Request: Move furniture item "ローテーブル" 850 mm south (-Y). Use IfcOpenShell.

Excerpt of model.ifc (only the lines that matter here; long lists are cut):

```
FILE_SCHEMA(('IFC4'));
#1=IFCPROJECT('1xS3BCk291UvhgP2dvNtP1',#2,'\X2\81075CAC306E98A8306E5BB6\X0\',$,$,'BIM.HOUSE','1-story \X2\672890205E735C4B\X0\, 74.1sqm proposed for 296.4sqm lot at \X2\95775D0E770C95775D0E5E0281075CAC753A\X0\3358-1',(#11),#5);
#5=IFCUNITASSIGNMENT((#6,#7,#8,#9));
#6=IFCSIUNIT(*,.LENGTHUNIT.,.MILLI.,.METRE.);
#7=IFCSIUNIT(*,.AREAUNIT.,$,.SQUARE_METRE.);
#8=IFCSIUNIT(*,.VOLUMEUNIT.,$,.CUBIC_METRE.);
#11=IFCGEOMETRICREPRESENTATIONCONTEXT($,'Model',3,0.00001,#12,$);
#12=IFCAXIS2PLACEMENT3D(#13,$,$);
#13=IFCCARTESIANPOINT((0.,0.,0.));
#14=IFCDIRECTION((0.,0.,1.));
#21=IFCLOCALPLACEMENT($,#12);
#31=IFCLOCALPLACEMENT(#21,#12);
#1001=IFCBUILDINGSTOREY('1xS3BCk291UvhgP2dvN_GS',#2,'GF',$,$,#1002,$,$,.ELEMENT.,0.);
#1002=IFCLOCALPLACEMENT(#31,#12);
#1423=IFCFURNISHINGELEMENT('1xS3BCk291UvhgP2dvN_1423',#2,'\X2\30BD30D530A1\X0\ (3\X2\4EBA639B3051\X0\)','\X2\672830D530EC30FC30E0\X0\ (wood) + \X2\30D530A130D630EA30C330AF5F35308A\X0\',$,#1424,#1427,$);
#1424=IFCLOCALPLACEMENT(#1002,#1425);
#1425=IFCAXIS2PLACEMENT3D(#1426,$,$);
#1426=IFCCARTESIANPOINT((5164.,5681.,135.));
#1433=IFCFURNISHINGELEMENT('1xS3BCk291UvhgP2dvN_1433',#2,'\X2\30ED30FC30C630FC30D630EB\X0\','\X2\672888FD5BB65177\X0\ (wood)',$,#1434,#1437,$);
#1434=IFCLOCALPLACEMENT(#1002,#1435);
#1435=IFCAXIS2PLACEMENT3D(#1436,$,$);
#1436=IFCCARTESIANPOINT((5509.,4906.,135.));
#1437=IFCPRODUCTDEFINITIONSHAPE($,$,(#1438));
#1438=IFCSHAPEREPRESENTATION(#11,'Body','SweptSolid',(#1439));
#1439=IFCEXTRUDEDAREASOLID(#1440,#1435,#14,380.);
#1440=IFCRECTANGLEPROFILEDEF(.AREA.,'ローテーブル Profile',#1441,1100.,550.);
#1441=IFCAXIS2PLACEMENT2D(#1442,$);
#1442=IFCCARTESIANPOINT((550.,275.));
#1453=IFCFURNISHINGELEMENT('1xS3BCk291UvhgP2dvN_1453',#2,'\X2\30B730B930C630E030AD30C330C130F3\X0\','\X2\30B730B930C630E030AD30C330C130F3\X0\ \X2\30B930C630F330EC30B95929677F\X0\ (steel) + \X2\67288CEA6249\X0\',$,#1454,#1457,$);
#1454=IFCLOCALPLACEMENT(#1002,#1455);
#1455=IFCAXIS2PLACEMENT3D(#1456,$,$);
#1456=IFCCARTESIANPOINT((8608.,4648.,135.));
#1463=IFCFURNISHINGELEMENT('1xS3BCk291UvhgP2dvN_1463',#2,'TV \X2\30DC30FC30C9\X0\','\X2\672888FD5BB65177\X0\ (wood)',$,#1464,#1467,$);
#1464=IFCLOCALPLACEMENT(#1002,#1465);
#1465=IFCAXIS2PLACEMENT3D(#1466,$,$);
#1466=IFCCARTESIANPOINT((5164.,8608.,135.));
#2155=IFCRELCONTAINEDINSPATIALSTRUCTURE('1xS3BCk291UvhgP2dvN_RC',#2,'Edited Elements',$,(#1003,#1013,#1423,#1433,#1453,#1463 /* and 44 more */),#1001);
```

```python
import ifcopenshell
import ifcopenshell.api.geometry
import ifcopenshell.util.placement
import ifcopenshell.util.unit

model = ifcopenshell.open("model.ifc")
unit_scale = ifcopenshell.util.unit.calculate_unit_scale(model)

item = model.by_guid("1xS3BCk291UvhgP2dvN_1433")
matrix = ifcopenshell.util.placement.get_local_placement(item.ObjectPlacement)
matrix[1, 3] -= 0.85 / unit_scale
ifcopenshell.api.geometry.edit_object_placement(model, product=item, matrix=matrix, is_si=False)

print(ifcopenshell.util.placement.get_local_placement(item.ObjectPlacement).round(3) + 0.0)

model.write("model_rev.ifc")
```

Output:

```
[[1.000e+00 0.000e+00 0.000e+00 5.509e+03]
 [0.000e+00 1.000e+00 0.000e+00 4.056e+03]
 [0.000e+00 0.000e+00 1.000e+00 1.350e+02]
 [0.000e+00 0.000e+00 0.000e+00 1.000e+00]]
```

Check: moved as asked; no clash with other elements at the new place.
